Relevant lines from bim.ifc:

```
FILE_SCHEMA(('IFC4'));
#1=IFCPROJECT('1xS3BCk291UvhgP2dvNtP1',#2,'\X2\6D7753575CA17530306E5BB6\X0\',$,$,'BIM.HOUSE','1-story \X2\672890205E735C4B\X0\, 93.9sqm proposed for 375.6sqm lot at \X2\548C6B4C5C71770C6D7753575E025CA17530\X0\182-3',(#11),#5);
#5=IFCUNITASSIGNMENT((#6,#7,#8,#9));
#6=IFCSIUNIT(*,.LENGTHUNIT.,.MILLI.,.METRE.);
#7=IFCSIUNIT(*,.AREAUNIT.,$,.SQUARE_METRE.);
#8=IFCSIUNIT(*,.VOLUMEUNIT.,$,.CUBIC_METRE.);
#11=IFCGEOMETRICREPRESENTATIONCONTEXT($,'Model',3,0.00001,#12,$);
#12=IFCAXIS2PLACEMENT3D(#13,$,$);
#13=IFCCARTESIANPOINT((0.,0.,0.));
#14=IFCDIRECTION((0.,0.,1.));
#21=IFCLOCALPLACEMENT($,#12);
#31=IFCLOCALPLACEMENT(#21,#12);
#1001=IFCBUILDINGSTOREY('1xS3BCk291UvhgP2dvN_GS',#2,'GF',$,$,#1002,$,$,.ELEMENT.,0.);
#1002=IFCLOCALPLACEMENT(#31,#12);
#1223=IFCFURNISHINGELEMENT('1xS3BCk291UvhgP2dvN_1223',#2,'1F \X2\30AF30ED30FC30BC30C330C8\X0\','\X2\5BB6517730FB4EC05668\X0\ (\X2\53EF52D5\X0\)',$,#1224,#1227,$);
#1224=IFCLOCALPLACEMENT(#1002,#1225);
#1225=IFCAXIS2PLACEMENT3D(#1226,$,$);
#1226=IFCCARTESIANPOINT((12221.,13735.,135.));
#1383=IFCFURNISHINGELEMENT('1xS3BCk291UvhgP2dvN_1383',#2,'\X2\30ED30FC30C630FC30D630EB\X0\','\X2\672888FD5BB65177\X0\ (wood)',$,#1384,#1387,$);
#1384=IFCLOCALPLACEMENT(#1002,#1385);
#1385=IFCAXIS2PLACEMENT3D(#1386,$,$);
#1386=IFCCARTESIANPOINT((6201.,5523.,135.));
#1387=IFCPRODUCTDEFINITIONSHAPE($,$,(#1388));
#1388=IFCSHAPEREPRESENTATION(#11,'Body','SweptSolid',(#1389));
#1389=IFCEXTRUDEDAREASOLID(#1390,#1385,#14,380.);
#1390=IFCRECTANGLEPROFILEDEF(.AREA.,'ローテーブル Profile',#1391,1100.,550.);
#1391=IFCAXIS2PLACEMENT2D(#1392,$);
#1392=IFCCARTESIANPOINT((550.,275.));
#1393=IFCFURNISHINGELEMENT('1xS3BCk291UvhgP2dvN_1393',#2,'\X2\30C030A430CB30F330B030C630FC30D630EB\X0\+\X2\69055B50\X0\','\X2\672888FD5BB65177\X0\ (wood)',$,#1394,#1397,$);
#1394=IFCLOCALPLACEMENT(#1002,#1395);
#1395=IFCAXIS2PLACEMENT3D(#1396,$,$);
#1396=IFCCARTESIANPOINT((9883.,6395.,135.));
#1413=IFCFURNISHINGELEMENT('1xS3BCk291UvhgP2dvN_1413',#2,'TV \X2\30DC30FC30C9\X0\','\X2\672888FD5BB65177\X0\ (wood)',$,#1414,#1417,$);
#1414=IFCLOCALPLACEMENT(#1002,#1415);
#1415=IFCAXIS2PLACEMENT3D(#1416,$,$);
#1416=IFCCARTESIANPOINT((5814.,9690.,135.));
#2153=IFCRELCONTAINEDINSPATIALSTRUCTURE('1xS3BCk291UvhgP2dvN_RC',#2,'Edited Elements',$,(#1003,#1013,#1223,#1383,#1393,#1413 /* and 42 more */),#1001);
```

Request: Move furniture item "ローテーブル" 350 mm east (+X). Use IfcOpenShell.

```python
import ifcopenshell
import ifcopenshell.api.geometry
import ifcopenshell.util.placement

model = ifcopenshell.open("bim.ifc")

item = model.by_guid("1xS3BCk291UvhgP2dvN_1383")
matrix = ifcopenshell.util.placement.get_local_placement(item.ObjectPlacement)
matrix[0, 3] += 350.0
ifcopenshell.api.geometry.edit_object_placement(model, product=item, matrix=matrix, is_si=False)

print(ifcopenshell.util.placement.get_local_placement(item.ObjectPlacement).round(3) + 0.0)

model.write("bim_rev.ifc")
```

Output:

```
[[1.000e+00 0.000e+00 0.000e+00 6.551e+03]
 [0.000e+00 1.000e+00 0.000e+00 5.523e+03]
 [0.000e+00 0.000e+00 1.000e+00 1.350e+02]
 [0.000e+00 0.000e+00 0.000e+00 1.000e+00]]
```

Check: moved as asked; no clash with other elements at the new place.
